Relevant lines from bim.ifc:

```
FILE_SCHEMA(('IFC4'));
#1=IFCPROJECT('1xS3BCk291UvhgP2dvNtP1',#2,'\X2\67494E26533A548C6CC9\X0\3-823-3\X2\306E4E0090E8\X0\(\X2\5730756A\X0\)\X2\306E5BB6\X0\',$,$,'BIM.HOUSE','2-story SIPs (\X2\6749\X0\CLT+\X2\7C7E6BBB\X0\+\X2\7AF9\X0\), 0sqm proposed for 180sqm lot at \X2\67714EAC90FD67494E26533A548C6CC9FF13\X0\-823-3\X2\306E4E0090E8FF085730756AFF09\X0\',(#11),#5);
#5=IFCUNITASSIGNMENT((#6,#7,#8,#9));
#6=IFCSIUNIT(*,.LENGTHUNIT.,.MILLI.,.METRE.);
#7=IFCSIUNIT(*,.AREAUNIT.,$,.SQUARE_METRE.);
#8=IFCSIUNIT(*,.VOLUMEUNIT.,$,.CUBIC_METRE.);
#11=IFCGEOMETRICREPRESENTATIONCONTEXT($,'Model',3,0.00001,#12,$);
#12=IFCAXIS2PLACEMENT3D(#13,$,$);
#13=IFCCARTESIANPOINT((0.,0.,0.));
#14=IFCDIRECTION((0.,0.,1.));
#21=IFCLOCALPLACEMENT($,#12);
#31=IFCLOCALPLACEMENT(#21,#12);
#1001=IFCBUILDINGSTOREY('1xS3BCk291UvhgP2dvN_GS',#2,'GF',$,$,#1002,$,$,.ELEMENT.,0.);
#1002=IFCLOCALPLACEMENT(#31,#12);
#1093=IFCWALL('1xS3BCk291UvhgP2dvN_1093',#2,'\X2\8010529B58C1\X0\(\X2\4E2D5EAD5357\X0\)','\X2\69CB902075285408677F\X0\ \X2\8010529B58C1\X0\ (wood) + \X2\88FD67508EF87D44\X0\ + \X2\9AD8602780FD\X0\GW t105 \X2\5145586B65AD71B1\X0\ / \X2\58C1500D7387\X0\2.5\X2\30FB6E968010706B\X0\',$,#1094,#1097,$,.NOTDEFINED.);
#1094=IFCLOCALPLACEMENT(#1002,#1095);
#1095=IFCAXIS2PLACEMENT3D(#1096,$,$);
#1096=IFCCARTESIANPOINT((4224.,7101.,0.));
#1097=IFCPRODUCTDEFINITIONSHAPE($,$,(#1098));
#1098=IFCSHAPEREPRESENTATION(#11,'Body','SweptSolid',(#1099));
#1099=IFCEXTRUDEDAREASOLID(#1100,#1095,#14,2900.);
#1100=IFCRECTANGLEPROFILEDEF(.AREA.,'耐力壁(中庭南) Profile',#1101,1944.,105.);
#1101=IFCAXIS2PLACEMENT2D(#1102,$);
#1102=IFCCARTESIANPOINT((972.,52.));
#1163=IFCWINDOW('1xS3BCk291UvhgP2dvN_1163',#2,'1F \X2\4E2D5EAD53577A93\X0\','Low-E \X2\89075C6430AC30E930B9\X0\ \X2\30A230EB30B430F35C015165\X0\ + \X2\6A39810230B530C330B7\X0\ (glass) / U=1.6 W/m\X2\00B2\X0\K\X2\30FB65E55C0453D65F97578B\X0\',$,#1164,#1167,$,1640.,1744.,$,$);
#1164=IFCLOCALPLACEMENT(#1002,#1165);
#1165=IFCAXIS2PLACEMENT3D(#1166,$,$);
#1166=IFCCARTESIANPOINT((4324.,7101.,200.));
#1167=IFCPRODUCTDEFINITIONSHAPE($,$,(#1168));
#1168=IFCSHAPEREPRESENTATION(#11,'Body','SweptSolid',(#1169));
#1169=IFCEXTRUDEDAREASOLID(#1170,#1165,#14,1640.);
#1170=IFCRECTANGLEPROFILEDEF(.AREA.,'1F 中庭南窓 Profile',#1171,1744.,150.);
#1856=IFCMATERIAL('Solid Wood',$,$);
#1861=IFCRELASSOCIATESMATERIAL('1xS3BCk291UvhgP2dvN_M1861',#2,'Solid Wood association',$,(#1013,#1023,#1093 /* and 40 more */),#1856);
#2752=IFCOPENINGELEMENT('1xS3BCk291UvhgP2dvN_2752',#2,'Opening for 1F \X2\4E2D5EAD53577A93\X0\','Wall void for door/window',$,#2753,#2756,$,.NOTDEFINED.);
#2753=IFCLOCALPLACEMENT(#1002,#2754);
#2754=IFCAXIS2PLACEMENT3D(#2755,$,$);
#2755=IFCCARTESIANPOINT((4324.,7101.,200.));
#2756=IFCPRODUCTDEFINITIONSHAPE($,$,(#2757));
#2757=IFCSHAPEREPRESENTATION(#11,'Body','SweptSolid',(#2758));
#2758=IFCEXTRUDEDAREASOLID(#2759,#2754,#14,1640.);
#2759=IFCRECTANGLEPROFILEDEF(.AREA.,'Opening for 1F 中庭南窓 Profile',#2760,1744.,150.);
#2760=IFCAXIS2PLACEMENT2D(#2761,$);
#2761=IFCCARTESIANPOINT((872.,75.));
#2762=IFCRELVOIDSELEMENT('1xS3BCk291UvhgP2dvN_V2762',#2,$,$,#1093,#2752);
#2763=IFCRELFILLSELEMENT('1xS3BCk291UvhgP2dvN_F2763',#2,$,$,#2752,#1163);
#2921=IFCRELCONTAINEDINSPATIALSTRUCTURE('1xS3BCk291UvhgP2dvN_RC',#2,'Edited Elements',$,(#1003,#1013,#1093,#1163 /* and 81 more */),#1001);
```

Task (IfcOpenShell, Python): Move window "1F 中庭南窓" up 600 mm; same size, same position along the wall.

```python
import numpy as np
import ifcopenshell
import ifcopenshell.api.geometry
import ifcopenshell.util.placement
import ifcopenshell.util.unit

model = ifcopenshell.open("bim.ifc")
unit_scale = ifcopenshell.util.unit.calculate_unit_scale(model)

window = model.by_guid("1xS3BCk291UvhgP2dvN_1163")
opening = window.FillsVoids[0].RelatingOpeningElement
dz = 600.0

shift = np.array([0.0, 0.0, dz])
# The window is not placed relative to its opening, so move both.
for product in (opening, window):
    matrix = ifcopenshell.util.placement.get_local_placement(product.ObjectPlacement)
    matrix[:3, 3] += shift
    ifcopenshell.api.geometry.edit_object_placement(model, product=product, matrix=matrix, is_si=False)

print(f"moved by {dz * unit_scale:+.3f} m")

model.write("bim_v2.ifc")
```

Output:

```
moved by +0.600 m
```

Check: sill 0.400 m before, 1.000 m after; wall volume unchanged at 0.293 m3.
